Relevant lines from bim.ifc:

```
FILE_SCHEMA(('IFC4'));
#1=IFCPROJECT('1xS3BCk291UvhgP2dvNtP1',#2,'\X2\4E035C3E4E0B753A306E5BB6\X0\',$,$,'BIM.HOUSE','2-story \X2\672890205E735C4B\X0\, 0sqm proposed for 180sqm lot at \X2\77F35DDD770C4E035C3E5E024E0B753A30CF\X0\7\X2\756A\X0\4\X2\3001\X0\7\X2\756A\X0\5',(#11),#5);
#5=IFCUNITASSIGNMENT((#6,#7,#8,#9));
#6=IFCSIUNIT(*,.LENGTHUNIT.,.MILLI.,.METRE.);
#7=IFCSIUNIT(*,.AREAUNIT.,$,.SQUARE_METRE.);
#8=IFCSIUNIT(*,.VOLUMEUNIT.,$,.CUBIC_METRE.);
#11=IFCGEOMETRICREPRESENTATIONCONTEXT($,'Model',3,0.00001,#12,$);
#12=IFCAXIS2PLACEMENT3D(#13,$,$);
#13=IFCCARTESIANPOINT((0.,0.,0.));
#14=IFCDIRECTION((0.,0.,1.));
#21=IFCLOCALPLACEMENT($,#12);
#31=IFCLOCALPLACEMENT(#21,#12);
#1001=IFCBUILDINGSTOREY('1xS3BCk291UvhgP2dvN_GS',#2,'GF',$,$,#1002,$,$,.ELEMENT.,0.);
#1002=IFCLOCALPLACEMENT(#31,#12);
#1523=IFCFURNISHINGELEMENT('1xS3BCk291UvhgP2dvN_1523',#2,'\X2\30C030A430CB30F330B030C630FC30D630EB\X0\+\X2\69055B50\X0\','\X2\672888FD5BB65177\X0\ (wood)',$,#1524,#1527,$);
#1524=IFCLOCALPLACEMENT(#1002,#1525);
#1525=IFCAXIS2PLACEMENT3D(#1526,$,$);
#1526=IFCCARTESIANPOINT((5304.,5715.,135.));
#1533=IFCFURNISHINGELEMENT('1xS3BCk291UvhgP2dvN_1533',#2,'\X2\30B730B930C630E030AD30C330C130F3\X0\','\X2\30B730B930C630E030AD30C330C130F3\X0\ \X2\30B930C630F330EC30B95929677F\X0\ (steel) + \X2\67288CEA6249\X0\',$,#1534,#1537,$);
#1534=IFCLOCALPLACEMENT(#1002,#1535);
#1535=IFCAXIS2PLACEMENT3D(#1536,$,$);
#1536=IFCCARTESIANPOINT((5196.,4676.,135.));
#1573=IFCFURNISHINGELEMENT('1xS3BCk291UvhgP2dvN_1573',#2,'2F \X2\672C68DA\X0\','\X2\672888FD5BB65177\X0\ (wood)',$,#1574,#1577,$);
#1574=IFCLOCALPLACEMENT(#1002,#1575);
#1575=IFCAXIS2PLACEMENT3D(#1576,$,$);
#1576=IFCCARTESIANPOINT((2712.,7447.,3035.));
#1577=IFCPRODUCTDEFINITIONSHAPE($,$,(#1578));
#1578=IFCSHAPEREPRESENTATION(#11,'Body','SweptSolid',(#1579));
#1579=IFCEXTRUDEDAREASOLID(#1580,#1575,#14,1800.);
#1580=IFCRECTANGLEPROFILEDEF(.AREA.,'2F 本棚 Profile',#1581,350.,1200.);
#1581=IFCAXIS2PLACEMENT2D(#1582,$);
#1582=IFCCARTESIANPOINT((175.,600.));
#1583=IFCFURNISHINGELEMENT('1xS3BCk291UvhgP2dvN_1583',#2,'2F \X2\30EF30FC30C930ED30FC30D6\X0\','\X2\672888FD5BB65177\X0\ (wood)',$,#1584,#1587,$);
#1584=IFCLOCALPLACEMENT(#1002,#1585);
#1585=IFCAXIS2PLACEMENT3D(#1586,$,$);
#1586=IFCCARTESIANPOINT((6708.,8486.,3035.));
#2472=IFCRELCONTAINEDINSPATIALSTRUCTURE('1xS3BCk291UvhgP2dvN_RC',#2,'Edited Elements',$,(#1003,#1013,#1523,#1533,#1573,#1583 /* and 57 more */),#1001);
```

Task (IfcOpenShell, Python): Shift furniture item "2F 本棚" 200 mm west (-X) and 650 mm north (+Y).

```python
import ifcopenshell
import ifcopenshell.api.geometry
import ifcopenshell.util.placement

model = ifcopenshell.open("bim.ifc")

item = model.by_guid("1xS3BCk291UvhgP2dvN_1573")
matrix = ifcopenshell.util.placement.get_local_placement(item.ObjectPlacement)
matrix[0, 3] -= 200.0
matrix[1, 3] += 650.0
ifcopenshell.api.geometry.edit_object_placement(model, product=item, matrix=matrix, is_si=False)

print(ifcopenshell.util.placement.get_local_placement(item.ObjectPlacement).round(3) + 0.0)

model.write("bim_updated.ifc")
```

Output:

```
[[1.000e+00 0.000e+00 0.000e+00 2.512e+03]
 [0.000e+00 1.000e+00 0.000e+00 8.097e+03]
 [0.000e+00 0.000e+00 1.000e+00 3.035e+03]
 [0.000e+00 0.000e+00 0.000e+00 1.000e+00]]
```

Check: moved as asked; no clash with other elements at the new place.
